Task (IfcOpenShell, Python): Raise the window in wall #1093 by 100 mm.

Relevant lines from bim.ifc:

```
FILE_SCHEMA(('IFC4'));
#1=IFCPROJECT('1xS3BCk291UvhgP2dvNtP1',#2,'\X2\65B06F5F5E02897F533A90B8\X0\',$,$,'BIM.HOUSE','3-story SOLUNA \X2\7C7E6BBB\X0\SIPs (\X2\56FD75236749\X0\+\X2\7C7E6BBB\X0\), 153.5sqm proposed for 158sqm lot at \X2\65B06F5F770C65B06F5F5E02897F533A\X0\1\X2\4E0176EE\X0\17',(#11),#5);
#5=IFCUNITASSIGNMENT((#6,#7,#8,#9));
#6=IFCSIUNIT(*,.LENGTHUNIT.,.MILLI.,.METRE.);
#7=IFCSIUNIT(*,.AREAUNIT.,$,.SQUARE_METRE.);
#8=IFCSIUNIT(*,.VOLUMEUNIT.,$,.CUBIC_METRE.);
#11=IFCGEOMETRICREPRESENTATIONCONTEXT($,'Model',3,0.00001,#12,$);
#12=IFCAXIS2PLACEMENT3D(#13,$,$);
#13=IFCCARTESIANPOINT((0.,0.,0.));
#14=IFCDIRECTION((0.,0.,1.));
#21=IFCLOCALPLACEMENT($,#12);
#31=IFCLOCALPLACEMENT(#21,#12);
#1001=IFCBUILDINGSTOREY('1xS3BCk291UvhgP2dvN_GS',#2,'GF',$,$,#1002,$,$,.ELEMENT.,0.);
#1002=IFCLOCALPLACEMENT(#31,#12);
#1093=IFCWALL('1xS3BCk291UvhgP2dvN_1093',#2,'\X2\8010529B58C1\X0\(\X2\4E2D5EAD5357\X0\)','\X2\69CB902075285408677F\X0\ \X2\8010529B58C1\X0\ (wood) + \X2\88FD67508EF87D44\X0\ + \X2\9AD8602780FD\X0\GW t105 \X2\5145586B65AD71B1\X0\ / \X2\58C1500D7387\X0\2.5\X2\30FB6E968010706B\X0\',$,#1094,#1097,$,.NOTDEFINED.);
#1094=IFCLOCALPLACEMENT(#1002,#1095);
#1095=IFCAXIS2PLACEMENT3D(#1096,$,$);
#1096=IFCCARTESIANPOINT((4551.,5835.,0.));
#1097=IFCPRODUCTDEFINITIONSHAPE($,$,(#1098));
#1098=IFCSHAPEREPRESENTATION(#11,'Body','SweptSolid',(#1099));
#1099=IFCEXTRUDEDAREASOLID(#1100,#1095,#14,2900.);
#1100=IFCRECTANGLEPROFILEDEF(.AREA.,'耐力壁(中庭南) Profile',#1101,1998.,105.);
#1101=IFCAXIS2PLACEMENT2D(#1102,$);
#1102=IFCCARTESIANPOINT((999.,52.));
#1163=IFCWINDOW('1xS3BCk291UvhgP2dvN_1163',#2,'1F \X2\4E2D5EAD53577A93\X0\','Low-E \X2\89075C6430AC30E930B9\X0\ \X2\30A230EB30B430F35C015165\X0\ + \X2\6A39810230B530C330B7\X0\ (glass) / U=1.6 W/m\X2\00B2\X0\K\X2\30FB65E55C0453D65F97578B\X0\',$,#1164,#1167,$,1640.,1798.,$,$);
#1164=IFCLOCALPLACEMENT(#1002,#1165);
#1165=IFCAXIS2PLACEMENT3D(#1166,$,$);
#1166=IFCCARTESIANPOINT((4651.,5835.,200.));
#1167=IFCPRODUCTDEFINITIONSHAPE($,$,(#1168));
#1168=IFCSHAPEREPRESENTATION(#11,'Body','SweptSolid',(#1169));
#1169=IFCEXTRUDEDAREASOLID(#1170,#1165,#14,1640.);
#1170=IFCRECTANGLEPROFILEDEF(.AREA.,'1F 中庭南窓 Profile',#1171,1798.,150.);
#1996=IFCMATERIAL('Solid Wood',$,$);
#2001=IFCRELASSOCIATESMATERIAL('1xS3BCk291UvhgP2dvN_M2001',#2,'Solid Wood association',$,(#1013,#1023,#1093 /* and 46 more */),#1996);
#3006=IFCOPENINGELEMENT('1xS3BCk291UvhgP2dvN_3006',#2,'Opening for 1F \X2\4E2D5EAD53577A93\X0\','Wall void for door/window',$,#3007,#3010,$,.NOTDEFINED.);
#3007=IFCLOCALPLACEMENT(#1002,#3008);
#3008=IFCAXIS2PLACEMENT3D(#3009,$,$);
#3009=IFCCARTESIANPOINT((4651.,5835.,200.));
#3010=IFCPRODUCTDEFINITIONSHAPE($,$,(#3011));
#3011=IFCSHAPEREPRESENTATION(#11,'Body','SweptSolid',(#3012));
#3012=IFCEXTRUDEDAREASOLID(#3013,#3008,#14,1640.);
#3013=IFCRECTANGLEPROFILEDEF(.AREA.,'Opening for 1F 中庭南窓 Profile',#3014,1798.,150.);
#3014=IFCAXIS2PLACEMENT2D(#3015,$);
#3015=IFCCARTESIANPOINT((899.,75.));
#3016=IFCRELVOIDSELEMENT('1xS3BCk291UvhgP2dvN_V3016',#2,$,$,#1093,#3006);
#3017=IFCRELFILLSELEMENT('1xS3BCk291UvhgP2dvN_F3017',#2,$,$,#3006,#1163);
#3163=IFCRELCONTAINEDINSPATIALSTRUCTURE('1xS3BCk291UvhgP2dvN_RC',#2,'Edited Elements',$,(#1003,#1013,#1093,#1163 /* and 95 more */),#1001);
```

```python
import numpy as np
import ifcopenshell
import ifcopenshell.api.geometry
import ifcopenshell.util.placement
import ifcopenshell.util.unit

model = ifcopenshell.open("bim.ifc")
unit_scale = ifcopenshell.util.unit.calculate_unit_scale(model)

window = model.by_id(1163)
opening = window.FillsVoids[0].RelatingOpeningElement
dz = 100.0

shift = np.array([0.0, 0.0, dz])
# The window is not placed relative to its opening, so move both.
for product in (opening, window):
    matrix = ifcopenshell.util.placement.get_local_placement(product.ObjectPlacement)
    matrix[:3, 3] += shift
    ifcopenshell.api.geometry.edit_object_placement(model, product=product, matrix=matrix, is_si=False)

print(f"moved by {dz * unit_scale:+.3f} m")

model.write("bim_edited.ifc")
```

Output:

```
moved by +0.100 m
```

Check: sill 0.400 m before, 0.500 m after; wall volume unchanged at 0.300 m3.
